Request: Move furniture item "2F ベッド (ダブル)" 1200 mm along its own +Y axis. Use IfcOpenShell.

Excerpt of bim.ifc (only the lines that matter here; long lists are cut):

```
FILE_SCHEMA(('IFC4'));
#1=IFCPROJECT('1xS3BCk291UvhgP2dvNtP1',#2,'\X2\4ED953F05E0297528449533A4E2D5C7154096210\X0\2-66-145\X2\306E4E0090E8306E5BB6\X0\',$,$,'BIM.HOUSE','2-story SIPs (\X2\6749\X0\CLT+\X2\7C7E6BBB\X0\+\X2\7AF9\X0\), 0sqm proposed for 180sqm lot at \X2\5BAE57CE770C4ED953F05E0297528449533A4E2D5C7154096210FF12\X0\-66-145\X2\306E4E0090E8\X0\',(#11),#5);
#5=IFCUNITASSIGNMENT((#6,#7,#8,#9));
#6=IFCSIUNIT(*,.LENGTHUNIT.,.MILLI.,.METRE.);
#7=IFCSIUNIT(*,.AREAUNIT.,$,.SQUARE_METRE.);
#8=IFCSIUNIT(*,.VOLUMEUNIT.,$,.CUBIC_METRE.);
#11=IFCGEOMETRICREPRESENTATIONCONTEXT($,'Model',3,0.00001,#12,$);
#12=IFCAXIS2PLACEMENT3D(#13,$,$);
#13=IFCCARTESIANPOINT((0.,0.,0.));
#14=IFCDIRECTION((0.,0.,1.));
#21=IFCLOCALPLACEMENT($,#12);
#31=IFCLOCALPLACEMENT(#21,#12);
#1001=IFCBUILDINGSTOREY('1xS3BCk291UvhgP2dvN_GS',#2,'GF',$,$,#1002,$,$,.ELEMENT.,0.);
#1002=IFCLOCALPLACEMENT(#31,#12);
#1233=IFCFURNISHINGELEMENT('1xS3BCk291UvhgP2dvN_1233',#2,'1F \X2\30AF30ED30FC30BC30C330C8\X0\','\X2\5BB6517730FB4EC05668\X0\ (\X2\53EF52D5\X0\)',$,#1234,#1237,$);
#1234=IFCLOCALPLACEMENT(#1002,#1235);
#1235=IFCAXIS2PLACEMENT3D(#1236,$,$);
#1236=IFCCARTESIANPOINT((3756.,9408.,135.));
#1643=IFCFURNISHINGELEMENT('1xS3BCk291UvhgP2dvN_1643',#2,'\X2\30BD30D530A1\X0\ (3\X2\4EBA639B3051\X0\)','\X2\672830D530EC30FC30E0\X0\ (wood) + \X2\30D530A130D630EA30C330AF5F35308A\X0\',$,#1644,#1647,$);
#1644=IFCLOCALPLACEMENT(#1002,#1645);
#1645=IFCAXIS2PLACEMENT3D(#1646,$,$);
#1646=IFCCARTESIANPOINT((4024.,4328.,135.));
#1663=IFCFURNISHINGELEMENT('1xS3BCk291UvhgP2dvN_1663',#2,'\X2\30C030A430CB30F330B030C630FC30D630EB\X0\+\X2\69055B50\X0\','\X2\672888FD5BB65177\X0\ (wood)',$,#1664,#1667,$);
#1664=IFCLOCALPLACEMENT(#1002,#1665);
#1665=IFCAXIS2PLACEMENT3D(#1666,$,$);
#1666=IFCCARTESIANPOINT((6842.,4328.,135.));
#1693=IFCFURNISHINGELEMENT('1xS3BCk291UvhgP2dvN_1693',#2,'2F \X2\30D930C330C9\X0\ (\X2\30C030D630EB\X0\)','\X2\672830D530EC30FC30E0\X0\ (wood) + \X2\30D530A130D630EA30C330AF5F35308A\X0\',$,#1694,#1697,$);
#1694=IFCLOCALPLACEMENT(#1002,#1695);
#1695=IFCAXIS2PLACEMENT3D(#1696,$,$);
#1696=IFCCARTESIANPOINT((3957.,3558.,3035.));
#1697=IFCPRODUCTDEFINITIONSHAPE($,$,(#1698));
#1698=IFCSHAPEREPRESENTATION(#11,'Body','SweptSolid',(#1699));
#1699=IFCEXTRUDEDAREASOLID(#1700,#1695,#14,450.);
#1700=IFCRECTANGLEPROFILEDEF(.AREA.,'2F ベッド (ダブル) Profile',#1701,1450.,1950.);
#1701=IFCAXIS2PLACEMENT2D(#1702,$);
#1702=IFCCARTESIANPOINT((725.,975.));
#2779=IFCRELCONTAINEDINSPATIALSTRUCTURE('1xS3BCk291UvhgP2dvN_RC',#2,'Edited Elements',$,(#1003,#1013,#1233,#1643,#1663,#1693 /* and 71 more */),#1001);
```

```python
import ifcopenshell
import ifcopenshell.api.geometry
import ifcopenshell.util.placement
import ifcopenshell.util.unit

model = ifcopenshell.open("bim.ifc")
unit_scale = ifcopenshell.util.unit.calculate_unit_scale(model)

item = model.by_guid("1xS3BCk291UvhgP2dvN_1693")
matrix = ifcopenshell.util.placement.get_local_placement(item.ObjectPlacement)
matrix[:3, 3] += matrix[:3, 1] * 1.2 / unit_scale
ifcopenshell.api.geometry.edit_object_placement(model, product=item, matrix=matrix, is_si=False)

print(ifcopenshell.util.placement.get_local_placement(item.ObjectPlacement).round(3) + 0.0)

model.write("bim_updated.ifc")
```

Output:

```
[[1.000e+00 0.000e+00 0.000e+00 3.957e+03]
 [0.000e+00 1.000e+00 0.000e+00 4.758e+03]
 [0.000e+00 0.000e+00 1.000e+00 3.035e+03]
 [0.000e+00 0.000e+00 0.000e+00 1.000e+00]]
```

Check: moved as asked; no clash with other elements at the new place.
